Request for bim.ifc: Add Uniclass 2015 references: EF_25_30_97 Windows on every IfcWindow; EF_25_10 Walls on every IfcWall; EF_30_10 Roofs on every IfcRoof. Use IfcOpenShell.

First a look at what the model holds.

```python
import ifcopenshell

model = ifcopenshell.open("bim.ifc")
print(model.schema)
print("classifications:", [c.Name for c in model.by_type("IfcClassification")])
for ifc_class in ("IfcDoor", "IfcRoof", "IfcStair", "IfcWall", "IfcWindow"):
    print(ifc_class, len(model.by_type(ifc_class)))
```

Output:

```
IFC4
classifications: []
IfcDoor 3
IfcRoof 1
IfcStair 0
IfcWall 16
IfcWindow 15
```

```python
import ifcopenshell
import ifcopenshell.api.classification

model = ifcopenshell.open("bim.ifc")

system = ifcopenshell.api.classification.add_classification(model, classification="Uniclass 2015")

codes = {
    "IfcWindow": ("EF_25_30_97", "Windows"),
    "IfcWall": ("EF_25_10", "Walls"),
    "IfcRoof": ("EF_30_10", "Roofs"),
}
for ifc_class, (code, name) in codes.items():
    products = model.by_type(ifc_class)
    ifcopenshell.api.classification.add_reference(
        model, products=products, classification=system, identification=code, name=name
    )
    print(code, len(products))

model.write("bim-out.ifc")
```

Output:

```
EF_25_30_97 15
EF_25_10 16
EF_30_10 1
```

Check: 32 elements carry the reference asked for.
